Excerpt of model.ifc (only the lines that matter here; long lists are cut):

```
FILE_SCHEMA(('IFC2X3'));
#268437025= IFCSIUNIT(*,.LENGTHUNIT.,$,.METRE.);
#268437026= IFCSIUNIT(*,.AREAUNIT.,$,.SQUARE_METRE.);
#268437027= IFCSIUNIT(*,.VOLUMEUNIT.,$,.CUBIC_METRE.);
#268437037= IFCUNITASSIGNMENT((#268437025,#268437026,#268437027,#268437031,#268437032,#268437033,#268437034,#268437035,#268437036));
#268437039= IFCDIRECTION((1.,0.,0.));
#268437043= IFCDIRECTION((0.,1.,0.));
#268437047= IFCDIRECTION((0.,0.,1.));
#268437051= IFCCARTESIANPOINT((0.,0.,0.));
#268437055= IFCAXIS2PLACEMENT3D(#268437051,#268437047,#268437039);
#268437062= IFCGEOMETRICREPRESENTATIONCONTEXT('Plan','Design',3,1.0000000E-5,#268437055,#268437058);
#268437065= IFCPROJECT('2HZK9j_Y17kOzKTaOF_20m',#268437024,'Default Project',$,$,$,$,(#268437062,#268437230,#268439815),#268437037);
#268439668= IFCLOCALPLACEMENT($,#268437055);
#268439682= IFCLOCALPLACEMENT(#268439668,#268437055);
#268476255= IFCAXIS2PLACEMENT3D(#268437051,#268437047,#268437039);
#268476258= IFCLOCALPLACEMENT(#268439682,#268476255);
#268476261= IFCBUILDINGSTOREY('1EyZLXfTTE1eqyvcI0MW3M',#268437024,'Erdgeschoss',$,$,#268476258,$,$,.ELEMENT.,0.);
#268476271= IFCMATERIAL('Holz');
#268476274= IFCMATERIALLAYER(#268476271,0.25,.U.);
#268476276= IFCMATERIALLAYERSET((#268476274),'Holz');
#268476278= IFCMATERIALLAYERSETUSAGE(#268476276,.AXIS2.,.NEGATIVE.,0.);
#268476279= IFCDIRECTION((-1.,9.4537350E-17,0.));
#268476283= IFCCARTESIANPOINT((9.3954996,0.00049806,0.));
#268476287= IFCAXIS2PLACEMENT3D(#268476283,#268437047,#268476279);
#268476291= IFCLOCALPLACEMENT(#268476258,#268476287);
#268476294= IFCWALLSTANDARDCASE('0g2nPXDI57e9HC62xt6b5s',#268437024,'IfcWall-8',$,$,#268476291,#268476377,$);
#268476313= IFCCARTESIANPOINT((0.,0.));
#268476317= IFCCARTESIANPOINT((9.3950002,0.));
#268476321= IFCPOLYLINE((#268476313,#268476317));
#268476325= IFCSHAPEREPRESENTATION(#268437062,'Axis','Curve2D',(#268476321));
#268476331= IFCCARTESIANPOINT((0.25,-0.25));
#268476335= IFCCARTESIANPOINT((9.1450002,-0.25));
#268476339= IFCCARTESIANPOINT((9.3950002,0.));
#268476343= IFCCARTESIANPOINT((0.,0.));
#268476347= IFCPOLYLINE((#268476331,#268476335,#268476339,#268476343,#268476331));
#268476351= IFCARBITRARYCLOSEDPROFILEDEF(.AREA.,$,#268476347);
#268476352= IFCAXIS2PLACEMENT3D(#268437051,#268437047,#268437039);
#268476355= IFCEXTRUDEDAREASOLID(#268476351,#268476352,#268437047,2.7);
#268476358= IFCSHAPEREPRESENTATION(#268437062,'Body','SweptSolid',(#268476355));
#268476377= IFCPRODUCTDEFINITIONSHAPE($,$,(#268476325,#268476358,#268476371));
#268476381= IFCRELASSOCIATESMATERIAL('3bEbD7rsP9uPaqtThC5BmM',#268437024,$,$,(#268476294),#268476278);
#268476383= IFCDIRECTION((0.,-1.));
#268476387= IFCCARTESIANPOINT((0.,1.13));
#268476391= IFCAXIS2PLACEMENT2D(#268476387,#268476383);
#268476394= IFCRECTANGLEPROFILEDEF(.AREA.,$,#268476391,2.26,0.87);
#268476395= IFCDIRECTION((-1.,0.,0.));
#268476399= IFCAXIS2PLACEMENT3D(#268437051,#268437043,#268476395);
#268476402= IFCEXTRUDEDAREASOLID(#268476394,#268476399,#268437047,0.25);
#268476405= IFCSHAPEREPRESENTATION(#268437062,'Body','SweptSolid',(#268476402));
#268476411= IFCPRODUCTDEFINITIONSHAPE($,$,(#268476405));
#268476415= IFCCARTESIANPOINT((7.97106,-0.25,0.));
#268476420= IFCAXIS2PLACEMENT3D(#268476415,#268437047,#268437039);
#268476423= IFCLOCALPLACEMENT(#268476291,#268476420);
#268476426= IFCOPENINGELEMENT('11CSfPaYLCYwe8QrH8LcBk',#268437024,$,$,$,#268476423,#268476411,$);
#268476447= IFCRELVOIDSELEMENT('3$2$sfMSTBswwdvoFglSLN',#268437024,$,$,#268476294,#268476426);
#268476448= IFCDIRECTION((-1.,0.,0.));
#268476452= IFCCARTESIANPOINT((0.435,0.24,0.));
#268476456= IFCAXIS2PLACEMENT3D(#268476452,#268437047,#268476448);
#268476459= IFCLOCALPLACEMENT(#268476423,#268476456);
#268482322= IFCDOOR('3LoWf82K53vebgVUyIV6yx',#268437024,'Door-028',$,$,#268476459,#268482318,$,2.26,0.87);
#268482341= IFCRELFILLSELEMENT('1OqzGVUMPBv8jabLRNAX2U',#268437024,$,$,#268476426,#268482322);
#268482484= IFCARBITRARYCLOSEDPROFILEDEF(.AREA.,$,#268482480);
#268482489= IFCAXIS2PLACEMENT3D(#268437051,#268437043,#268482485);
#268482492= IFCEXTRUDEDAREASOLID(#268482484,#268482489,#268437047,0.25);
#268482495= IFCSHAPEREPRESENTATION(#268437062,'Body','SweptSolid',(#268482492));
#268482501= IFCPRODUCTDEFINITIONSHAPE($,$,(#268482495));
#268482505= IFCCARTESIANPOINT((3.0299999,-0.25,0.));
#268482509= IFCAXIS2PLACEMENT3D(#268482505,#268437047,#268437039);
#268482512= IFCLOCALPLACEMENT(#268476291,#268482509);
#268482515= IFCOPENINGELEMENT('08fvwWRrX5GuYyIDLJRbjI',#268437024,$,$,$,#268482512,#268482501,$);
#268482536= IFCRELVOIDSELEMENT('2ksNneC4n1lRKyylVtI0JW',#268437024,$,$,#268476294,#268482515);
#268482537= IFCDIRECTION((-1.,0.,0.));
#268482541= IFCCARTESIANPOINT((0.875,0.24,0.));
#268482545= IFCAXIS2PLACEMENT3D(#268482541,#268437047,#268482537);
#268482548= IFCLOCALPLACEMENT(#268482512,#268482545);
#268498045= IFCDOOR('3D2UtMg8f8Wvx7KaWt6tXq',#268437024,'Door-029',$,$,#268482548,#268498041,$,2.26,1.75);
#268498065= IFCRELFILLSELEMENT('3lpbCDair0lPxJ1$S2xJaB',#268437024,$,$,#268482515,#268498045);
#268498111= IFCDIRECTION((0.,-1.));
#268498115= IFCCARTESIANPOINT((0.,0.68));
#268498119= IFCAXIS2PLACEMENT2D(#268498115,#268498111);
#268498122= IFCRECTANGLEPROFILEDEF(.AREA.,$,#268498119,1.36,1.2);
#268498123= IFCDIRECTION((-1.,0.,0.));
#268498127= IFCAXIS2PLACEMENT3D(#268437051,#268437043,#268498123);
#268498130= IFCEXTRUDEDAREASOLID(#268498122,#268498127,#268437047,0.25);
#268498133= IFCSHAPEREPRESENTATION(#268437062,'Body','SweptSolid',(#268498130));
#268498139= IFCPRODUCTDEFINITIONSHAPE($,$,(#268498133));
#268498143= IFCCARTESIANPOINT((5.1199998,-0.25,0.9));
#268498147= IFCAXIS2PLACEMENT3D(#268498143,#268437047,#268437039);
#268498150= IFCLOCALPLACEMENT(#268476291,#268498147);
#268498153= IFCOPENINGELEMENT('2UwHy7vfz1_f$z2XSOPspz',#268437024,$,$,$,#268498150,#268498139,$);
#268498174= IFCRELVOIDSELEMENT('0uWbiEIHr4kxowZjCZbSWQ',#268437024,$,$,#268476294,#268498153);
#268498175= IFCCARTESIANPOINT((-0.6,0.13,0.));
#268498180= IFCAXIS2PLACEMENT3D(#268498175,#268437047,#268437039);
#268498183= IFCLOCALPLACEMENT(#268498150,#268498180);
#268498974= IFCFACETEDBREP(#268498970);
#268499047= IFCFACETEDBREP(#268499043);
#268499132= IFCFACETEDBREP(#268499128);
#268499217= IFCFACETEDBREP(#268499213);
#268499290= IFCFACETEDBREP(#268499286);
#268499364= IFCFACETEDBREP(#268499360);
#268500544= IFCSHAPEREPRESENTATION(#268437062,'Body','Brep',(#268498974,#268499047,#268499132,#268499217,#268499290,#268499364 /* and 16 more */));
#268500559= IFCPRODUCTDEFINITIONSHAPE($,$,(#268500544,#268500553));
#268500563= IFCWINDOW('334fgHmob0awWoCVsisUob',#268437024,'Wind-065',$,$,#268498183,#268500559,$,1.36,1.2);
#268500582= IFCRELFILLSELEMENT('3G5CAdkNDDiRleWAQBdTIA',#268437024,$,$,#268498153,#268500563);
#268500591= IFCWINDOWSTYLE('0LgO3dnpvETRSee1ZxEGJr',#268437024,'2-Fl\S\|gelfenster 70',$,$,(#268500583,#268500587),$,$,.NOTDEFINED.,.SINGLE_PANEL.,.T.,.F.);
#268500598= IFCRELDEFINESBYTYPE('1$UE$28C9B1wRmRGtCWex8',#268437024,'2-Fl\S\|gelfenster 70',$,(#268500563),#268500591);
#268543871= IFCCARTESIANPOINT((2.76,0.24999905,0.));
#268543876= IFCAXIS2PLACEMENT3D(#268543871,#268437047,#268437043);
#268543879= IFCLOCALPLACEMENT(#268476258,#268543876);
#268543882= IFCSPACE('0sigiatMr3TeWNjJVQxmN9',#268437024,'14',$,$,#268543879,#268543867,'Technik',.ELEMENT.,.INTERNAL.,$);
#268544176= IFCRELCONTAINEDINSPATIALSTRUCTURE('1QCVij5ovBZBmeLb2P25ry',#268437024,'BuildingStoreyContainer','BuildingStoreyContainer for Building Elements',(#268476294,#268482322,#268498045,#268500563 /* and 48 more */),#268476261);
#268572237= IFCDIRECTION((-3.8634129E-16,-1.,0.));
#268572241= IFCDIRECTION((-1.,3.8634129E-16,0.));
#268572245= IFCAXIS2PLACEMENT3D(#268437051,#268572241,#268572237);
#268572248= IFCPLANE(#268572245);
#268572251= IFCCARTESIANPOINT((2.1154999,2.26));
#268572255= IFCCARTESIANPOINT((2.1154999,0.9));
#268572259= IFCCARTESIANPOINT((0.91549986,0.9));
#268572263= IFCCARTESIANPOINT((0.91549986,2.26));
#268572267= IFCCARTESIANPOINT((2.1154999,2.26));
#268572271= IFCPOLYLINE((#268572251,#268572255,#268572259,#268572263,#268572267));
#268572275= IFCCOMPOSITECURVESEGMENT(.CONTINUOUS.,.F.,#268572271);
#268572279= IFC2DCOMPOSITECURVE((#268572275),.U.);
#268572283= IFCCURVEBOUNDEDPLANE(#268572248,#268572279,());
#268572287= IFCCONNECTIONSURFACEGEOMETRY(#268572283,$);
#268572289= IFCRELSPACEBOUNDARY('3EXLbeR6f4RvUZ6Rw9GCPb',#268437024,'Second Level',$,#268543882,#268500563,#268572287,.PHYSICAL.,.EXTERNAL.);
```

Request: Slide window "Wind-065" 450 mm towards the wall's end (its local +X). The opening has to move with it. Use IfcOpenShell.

```python
import numpy as np
import ifcopenshell
import ifcopenshell.api.geometry
import ifcopenshell.util.placement
import ifcopenshell.util.unit

model = ifcopenshell.open("model.ifc")
unit_scale = ifcopenshell.util.unit.calculate_unit_scale(model)

window = model.by_guid("334fgHmob0awWoCVsisUob")
opening = window.FillsVoids[0].RelatingOpeningElement
wall = opening.VoidsElements[0].RelatingBuildingElement

wall_matrix = ifcopenshell.util.placement.get_local_placement(wall.ObjectPlacement)
shift = wall_matrix[:3, 0] * 0.45 / unit_scale
before = ifcopenshell.util.placement.get_local_placement(window.ObjectPlacement)[:3, 3].copy()

# The window is placed relative to its opening, so it follows when the opening moves.
matrix = ifcopenshell.util.placement.get_local_placement(opening.ObjectPlacement)
matrix[:3, 3] += shift
ifcopenshell.api.geometry.edit_object_placement(
    model, product=opening, matrix=matrix, is_si=False, should_transform_children=True
)

# Space boundary surfaces are stored in each space's coordinates; move them too.
for rel in window.ProvidesBoundaries:
    if not rel.ConnectionGeometry:
        continue
    surface = rel.ConnectionGeometry.SurfaceOnRelatingElement.BasisSurface
    space_matrix = ifcopenshell.util.placement.get_local_placement(rel.RelatingSpace.ObjectPlacement)
    point = np.array(surface.Position.Location.Coordinates) + space_matrix[:3, :3].T @ shift
    surface.Position = model.createIfcAxis2Placement3D(
        model.createIfcCartesianPoint(point.tolist()), surface.Position.Axis, surface.Position.RefDirection
    )

after = ifcopenshell.util.placement.get_local_placement(window.ObjectPlacement)[:3, 3]
print("window moved by", (after - before).round(3) + 0.0)

model.write("model_updated.ifc")
```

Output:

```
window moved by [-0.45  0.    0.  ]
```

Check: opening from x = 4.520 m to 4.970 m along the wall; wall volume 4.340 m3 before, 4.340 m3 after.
